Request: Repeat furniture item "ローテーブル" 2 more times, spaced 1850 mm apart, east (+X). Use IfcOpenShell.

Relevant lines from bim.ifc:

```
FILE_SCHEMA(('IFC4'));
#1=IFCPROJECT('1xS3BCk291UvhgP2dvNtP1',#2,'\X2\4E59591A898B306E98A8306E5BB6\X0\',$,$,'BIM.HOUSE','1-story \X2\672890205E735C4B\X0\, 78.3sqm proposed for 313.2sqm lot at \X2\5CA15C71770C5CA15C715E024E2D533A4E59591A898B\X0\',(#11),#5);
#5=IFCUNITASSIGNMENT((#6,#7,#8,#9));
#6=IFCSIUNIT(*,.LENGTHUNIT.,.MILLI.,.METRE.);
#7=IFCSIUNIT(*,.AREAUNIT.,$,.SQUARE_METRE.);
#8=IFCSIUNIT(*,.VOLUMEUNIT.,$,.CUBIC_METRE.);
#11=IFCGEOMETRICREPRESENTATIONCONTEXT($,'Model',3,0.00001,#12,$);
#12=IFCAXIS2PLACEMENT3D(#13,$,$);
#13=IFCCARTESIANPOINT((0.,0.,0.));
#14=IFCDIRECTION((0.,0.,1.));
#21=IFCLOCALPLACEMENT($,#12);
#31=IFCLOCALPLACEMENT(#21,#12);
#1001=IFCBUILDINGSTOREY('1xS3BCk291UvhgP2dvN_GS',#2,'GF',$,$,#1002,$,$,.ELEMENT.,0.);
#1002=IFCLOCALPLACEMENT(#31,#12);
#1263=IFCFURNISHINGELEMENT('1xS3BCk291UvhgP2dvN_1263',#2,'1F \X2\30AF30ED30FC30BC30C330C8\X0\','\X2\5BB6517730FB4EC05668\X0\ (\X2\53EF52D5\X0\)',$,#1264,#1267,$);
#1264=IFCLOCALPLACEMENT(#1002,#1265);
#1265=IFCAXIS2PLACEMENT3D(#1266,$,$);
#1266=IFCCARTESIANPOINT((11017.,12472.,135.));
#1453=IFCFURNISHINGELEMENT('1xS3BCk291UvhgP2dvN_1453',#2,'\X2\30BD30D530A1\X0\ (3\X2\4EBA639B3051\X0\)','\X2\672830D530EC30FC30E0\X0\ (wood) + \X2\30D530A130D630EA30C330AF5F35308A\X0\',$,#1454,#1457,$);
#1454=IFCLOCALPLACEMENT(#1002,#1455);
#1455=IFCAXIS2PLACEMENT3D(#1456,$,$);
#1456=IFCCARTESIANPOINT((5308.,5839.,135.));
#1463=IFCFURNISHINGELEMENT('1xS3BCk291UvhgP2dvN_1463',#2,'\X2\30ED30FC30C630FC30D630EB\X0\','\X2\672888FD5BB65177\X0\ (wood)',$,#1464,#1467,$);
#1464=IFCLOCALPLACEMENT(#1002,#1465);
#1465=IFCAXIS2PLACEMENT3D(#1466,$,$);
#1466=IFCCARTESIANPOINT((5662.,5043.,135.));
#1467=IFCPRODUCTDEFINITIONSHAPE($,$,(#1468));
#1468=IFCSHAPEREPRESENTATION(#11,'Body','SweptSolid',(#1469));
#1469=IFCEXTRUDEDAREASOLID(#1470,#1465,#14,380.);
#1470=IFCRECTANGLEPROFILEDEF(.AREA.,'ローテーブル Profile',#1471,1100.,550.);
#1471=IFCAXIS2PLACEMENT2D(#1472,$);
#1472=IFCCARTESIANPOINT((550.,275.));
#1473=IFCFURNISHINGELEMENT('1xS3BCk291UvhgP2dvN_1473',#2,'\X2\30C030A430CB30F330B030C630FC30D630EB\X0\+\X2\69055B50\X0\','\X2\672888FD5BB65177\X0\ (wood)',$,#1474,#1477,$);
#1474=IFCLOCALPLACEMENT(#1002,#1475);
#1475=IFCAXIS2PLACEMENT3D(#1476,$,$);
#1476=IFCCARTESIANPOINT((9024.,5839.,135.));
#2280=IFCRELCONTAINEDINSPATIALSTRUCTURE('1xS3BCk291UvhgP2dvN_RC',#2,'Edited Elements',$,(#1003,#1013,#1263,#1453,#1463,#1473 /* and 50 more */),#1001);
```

```python
import numpy as np
import ifcopenshell
import ifcopenshell.api.geometry
import ifcopenshell.api.root
import ifcopenshell.util.element
import ifcopenshell.util.placement
import ifcopenshell.util.unit

model = ifcopenshell.open("bim.ifc")
unit_scale = ifcopenshell.util.unit.calculate_unit_scale(model)


def reuse_history(source, copy):
    """copy_class also copies each property set's owner history, people and application; keep the originals."""
    for rel in copy.IsDefinedBy:
        if rel.is_a("IfcRelDefinesByProperties") and (history := rel.RelatingPropertyDefinition.OwnerHistory):
            rel.RelatingPropertyDefinition.OwnerHistory = source.OwnerHistory
            ifcopenshell.util.element.remove_deep2(model, history)


source = model.by_id(1463)
base = ifcopenshell.util.placement.get_local_placement(source.ObjectPlacement)
step = np.array([1.0, 0.0, 0.0]) * 1.85 / unit_scale

for i in range(1, 3):
    copy = ifcopenshell.api.root.copy_class(model, product=source)
    copy.Representation = ifcopenshell.util.element.copy_deep(
        model, source.Representation, exclude=["IfcGeometricRepresentationContext", "IfcRepresentationMap"]
    )
    reuse_history(source, copy)
    matrix = base.copy()
    matrix[:3, 3] += i * step
    print("added at", matrix[:3, 3].round(3) + 0.0)
    ifcopenshell.api.geometry.edit_object_placement(model, product=copy, matrix=matrix, is_si=False)

model.write("bim_v2.ifc")
```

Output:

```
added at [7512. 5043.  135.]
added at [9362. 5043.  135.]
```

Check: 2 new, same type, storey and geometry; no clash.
